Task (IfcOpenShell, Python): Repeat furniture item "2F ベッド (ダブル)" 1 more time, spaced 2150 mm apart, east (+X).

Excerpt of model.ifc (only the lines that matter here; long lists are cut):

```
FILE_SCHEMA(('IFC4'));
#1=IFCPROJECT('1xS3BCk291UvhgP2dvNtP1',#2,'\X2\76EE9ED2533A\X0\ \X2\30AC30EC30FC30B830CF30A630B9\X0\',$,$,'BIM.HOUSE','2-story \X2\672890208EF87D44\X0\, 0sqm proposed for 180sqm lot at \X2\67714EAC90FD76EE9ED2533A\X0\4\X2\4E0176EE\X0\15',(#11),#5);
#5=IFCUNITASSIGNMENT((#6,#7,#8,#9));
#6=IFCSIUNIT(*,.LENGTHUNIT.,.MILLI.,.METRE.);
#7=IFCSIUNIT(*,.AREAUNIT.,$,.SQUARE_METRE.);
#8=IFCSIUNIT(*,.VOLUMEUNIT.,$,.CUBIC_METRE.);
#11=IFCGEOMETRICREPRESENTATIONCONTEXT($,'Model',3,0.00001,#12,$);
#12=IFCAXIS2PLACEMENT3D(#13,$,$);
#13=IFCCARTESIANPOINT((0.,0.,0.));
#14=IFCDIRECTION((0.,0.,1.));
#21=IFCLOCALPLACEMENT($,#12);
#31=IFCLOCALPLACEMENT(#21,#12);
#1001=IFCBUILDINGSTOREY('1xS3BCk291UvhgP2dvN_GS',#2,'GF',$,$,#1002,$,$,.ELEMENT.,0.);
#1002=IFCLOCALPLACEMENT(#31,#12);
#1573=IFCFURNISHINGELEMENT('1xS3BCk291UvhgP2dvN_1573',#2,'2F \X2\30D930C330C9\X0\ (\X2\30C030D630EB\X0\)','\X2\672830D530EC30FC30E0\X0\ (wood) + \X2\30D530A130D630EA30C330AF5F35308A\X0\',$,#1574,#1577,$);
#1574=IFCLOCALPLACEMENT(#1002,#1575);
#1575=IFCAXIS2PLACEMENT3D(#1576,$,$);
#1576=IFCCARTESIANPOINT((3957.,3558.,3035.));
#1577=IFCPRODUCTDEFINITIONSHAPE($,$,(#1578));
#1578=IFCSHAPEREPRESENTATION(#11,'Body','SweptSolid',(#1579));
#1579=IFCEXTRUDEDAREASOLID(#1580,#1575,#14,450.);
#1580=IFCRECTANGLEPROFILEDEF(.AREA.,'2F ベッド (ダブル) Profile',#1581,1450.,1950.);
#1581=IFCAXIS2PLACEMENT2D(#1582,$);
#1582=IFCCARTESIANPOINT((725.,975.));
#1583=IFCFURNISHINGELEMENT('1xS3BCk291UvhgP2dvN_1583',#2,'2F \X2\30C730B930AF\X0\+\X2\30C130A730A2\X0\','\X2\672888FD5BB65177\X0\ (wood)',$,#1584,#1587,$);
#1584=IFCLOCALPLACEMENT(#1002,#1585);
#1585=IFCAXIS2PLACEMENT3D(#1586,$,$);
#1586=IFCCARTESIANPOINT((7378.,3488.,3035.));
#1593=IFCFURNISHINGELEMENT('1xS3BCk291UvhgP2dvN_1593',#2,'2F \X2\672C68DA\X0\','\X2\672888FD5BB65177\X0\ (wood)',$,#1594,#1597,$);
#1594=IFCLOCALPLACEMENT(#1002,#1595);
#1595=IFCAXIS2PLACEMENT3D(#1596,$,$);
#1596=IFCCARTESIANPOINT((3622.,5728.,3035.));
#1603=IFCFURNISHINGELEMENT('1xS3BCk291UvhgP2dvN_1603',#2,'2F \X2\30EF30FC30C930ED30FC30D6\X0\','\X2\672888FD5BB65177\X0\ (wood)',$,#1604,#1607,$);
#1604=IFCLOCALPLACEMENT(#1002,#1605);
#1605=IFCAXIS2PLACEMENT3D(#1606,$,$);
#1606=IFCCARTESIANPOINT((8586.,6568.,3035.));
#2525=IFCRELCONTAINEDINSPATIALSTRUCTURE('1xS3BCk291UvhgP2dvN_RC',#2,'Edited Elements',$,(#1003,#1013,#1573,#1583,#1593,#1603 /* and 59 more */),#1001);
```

```python
import numpy as np
import ifcopenshell
import ifcopenshell.api.geometry
import ifcopenshell.api.root
import ifcopenshell.util.element
import ifcopenshell.util.placement

model = ifcopenshell.open("model.ifc")


def reuse_history(source, copy):
    """copy_class also copies each property set's owner history, people and application; keep the originals."""
    for rel in copy.IsDefinedBy:
        if rel.is_a("IfcRelDefinesByProperties") and (history := rel.RelatingPropertyDefinition.OwnerHistory):
            rel.RelatingPropertyDefinition.OwnerHistory = source.OwnerHistory
            ifcopenshell.util.element.remove_deep2(model, history)


source = model.by_guid("1xS3BCk291UvhgP2dvN_1573")
base = ifcopenshell.util.placement.get_local_placement(source.ObjectPlacement)
step = np.array([1.0, 0.0, 0.0]) * 2150.0

for i in range(1, 2):
    copy = ifcopenshell.api.root.copy_class(model, product=source)
    copy.Representation = ifcopenshell.util.element.copy_deep(
        model, source.Representation, exclude=["IfcGeometricRepresentationContext", "IfcRepresentationMap"]
    )
    reuse_history(source, copy)
    matrix = base.copy()
    matrix[:3, 3] += i * step
    print("added at", matrix[:3, 3].round(3) + 0.0)
    ifcopenshell.api.geometry.edit_object_placement(model, product=copy, matrix=matrix, is_si=False)

model.write("model_edited.ifc")
```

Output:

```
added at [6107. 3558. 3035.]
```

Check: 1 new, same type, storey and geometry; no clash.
